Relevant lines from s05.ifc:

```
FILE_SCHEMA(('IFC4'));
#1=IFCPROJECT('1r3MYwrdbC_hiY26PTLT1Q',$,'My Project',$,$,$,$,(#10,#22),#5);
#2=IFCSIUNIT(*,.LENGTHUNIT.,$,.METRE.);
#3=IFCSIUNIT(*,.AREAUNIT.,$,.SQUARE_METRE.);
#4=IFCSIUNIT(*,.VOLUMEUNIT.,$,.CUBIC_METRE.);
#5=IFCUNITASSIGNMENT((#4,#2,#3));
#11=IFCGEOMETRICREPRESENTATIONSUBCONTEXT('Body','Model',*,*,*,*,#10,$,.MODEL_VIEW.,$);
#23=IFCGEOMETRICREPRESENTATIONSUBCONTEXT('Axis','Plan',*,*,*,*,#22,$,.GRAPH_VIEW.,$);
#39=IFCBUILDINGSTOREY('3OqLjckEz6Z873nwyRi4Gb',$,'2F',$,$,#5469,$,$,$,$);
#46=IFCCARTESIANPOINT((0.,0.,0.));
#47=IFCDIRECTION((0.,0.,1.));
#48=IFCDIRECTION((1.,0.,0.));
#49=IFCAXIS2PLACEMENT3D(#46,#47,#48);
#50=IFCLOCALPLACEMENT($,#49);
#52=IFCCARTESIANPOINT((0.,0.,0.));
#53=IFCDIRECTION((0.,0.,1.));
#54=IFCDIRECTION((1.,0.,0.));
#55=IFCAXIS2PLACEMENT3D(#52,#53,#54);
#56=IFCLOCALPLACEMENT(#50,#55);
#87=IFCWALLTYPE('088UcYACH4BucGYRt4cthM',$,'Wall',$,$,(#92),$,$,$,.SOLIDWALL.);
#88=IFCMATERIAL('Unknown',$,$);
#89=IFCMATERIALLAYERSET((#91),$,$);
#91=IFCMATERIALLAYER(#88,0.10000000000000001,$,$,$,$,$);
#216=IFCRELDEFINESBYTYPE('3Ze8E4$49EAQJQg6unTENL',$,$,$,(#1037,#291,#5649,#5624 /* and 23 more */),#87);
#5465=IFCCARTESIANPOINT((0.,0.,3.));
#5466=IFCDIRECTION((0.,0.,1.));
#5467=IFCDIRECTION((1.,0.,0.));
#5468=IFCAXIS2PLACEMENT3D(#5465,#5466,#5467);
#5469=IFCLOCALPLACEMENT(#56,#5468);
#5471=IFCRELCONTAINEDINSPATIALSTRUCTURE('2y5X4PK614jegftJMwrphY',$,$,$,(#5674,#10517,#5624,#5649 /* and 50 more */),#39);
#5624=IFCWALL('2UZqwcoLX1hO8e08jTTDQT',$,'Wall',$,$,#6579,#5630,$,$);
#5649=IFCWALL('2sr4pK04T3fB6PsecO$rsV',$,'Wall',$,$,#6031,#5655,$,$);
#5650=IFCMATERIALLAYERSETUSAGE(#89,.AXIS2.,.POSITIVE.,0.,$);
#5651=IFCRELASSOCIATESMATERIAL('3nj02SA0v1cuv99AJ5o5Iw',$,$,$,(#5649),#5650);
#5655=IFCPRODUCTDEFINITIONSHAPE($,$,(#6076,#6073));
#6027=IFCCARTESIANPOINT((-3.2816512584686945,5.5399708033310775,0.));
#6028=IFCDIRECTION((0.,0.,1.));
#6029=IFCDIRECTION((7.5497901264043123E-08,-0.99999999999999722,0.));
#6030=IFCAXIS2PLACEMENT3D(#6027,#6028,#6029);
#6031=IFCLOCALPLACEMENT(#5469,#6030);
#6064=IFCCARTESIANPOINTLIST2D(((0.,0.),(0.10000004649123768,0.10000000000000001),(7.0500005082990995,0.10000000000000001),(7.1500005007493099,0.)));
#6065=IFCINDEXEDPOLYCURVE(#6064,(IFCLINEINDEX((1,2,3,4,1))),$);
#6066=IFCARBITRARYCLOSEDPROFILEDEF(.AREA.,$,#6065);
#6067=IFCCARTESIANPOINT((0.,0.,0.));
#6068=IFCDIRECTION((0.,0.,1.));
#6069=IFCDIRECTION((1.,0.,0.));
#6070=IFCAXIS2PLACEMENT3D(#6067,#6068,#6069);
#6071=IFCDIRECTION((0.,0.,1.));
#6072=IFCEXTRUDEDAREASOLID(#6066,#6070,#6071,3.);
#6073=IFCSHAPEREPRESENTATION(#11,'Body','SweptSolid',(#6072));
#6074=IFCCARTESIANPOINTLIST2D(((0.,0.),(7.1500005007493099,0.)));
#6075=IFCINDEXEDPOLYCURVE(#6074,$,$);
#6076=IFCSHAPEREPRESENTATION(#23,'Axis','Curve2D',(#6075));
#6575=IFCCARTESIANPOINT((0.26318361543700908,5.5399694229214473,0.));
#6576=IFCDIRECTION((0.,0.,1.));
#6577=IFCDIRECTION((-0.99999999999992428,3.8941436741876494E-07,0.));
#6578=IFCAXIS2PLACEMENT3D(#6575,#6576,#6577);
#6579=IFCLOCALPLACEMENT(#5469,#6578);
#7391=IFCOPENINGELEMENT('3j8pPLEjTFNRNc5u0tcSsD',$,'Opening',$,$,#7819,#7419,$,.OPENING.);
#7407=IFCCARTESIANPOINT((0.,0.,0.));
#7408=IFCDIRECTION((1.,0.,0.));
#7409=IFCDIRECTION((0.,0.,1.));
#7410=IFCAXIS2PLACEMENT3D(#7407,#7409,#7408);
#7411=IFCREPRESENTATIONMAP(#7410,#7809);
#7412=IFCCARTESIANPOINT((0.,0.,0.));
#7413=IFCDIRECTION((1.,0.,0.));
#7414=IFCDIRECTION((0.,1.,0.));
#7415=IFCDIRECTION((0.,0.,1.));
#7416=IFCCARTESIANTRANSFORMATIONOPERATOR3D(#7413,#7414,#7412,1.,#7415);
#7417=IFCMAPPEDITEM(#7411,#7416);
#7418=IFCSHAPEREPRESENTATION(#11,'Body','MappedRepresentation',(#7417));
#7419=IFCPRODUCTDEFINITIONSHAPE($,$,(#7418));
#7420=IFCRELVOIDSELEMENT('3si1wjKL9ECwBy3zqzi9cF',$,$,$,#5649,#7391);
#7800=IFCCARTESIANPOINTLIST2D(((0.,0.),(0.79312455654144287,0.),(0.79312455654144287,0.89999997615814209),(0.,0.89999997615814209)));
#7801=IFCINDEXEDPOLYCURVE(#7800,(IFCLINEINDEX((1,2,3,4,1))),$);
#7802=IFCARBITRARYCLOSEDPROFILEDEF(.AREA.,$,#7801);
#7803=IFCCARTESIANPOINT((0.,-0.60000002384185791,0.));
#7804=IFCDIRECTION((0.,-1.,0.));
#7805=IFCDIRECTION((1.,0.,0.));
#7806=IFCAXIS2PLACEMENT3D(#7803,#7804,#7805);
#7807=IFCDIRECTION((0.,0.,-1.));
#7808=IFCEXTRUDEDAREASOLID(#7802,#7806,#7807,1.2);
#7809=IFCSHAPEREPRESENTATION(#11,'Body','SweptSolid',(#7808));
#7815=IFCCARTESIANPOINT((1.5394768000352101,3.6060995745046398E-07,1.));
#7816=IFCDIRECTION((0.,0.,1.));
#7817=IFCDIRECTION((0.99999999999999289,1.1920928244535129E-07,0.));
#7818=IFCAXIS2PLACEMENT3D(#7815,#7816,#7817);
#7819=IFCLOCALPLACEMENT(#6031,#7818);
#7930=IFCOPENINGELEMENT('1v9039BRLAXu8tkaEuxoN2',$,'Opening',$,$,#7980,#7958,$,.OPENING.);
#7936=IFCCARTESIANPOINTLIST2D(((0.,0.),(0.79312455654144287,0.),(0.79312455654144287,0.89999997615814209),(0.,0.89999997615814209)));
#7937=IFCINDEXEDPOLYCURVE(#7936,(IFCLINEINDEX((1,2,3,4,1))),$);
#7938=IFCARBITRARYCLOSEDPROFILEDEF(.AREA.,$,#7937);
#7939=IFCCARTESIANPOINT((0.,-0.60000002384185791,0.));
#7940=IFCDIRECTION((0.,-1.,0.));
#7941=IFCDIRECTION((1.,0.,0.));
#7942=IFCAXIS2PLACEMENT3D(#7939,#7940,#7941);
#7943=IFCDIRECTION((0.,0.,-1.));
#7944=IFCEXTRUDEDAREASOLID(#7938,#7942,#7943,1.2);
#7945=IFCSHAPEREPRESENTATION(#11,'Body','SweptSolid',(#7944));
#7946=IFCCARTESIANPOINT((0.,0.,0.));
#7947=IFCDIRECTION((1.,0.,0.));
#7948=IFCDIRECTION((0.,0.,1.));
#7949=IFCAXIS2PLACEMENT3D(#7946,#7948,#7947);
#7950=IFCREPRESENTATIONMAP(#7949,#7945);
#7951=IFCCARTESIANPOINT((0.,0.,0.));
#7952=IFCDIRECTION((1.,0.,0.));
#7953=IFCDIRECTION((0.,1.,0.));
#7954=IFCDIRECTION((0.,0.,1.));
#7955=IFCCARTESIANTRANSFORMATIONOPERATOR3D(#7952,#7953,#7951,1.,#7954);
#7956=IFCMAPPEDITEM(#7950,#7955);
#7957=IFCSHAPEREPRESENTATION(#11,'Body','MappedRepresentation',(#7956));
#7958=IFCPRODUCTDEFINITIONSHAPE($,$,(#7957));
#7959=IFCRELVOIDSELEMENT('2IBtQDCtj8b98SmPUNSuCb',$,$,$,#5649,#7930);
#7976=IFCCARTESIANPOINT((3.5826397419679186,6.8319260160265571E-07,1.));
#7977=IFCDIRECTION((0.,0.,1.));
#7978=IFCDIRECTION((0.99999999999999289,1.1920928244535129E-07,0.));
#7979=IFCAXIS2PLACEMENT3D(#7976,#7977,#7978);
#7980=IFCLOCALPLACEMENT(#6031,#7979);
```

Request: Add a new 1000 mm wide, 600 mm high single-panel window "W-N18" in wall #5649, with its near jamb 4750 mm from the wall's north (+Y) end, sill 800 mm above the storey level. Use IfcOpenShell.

```python
import numpy as np
import ifcopenshell
import ifcopenshell.api.feature
import ifcopenshell.api.geometry
import ifcopenshell.api.root
import ifcopenshell.api.spatial
import ifcopenshell.geom
import ifcopenshell.util.element
import ifcopenshell.util.placement
import ifcopenshell.util.representation
import ifcopenshell.util.shape
import ifcopenshell.util.unit

model = ifcopenshell.open("s05.ifc")
unit_scale = ifcopenshell.util.unit.calculate_unit_scale(model)
settings = ifcopenshell.geom.settings()


def volume(element):
    """Net volume in cubic metres, openings subtracted."""
    shape = ifcopenshell.geom.create_shape(settings, element)
    return ifcopenshell.util.shape.get_volume(shape.geometry)


wall = model.by_guid("2sr4pK04T3fB6PsecO$rsV")
storey = ifcopenshell.util.element.get_container(wall, ifc_class="IfcBuildingStorey")
context = ifcopenshell.util.representation.get_context(model, "Model", "Body", "MODEL_VIEW")
before = volume(wall)

width, height, from_end, sill = 1, 0.6, 4.75, 0.8  # metres

# The wall runs along its own X axis, and the end named is its -X end.
wall_shape = ifcopenshell.geom.create_shape(settings, wall)
x, y, z = ifcopenshell.util.shape.get_vertices(wall_shape.geometry).T
start = x.min() + from_end
face, thickness = float(y.min()), float(y.max() - y.min())
wall_matrix = ifcopenshell.util.placement.get_local_placement(wall.ObjectPlacement)
level = ifcopenshell.util.placement.get_local_placement(storey.ObjectPlacement)[2, 3]


def in_wall(x, y):
    """Placement at x, y metres in the wall's axes, at sill height."""
    matrix = wall_matrix.copy()
    matrix[:, 3] = wall_matrix @ np.array([x / unit_scale, y / unit_scale, 0.0, 1.0])
    matrix[2, 3] = level + sill / unit_scale
    return matrix


# Opening: a box that overshoots both wall faces by 50 mm.
opening = ifcopenshell.api.root.create_entity(model, ifc_class="IfcOpeningElement", predefined_type="OPENING")
box = ifcopenshell.api.geometry.add_wall_representation(
    model, context=context, length=width, height=height, thickness=thickness + 0.1
)
ifcopenshell.api.geometry.assign_representation(model, product=opening, representation=box)
ifcopenshell.api.geometry.edit_object_placement(model, product=opening, matrix=in_wall(start, face - 0.05), is_si=False)
ifcopenshell.api.feature.add_feature(model, feature=opening, element=wall)

window = ifcopenshell.api.root.create_entity(model, ifc_class="IfcWindow", name="W-N18", predefined_type="WINDOW")
window.OverallWidth, window.OverallHeight = width / unit_scale, height / unit_scale
window.PartitioningType = "SINGLE_PANEL"
body = ifcopenshell.api.geometry.add_window_representation(
    model,
    context=context,
    overall_width=window.OverallWidth,
    overall_height=window.OverallHeight,
    partition_type="SINGLE_PANEL",
)
ifcopenshell.api.geometry.assign_representation(model, product=window, representation=body)
ifcopenshell.api.spatial.assign_container(model, products=[window], relating_structure=storey)
ifcopenshell.api.feature.add_filling(model, opening=opening, element=window)

# Centre the window in the wall's thickness.
ifcopenshell.api.geometry.edit_object_placement(model, product=window, matrix=in_wall(start, face), is_si=False)
window_shape = ifcopenshell.geom.create_shape(settings, window)
depth = ifcopenshell.util.shape.get_vertices(window_shape.geometry)[:, 1]
offset = face + thickness / 2 - (depth.min() + depth.max()) / 2
ifcopenshell.api.geometry.edit_object_placement(model, product=window, matrix=in_wall(start, offset), is_si=False)

after = volume(wall)

print(f"wall volume {before:.3f} -> {after:.3f} m3")

model.write("s05-out.ifc")
```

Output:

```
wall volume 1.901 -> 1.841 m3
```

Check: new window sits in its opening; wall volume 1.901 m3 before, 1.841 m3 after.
